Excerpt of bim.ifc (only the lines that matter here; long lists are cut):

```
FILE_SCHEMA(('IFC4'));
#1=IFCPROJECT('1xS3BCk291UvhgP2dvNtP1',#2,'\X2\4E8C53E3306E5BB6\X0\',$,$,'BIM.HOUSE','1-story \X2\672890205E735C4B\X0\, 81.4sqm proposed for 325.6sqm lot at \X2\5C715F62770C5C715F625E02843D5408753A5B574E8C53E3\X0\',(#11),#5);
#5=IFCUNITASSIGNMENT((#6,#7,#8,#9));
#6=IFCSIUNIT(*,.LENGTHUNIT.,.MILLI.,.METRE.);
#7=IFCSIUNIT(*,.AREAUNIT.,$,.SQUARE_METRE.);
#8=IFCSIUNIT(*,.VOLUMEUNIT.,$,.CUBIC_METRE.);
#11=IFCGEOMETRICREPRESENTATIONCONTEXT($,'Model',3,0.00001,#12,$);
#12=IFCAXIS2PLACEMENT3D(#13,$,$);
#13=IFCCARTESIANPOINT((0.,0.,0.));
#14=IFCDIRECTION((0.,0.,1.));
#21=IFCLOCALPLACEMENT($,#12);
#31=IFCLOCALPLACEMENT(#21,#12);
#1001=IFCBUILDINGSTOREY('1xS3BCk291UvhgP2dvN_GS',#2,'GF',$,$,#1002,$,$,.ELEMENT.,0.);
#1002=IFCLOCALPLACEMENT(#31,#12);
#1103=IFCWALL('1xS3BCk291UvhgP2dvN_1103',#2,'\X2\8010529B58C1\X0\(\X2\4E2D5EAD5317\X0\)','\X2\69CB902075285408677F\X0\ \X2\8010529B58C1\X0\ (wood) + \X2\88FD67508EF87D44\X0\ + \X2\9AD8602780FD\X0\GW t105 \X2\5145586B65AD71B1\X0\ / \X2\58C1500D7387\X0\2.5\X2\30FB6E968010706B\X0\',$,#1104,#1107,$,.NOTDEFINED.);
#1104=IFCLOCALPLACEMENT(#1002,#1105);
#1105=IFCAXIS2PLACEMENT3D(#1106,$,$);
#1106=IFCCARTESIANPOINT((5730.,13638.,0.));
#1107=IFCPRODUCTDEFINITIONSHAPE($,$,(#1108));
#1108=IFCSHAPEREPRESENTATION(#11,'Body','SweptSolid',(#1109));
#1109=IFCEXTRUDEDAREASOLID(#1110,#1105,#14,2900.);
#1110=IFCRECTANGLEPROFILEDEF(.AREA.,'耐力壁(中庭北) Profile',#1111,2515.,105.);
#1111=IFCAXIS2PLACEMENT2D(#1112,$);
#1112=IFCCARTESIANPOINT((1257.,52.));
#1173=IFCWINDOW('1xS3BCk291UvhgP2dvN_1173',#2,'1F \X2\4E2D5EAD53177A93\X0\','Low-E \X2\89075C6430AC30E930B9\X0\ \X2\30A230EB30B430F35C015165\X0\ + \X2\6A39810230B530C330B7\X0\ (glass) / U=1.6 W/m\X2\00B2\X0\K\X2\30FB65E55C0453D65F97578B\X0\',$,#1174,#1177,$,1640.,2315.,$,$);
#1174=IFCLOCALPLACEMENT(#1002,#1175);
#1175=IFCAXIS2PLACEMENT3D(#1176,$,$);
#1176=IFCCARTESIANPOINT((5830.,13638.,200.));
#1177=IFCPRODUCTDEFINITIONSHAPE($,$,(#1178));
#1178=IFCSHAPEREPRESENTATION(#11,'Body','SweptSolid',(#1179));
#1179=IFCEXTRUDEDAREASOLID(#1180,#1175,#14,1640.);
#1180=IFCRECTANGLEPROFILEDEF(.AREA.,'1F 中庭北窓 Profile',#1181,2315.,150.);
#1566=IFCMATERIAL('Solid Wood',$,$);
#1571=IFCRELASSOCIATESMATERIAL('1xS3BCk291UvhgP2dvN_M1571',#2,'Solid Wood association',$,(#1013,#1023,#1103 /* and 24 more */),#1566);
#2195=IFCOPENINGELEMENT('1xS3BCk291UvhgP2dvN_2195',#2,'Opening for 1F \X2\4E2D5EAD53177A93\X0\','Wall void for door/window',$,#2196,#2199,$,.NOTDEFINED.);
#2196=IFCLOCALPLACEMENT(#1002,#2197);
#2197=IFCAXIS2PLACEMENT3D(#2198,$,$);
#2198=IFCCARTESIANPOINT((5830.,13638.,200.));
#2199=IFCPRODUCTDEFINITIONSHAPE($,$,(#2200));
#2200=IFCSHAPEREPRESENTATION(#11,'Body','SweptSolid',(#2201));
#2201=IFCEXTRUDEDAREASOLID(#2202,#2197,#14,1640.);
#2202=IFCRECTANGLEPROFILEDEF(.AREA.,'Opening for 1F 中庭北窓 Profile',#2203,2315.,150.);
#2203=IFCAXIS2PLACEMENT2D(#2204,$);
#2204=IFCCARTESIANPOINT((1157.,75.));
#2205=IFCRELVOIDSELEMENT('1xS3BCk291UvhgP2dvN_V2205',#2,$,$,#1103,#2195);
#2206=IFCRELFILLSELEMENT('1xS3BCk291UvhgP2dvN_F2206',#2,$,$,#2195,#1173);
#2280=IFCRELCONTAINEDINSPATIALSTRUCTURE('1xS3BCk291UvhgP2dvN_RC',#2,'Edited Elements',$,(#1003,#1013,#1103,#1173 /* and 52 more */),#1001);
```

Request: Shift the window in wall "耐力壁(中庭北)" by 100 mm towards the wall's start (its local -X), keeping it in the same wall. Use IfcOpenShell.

```python
import ifcopenshell
import ifcopenshell.api.geometry
import ifcopenshell.util.placement

model = ifcopenshell.open("bim.ifc")

window = model.by_guid("1xS3BCk291UvhgP2dvN_1173")
opening = window.FillsVoids[0].RelatingOpeningElement
wall = opening.VoidsElements[0].RelatingBuildingElement

wall_matrix = ifcopenshell.util.placement.get_local_placement(wall.ObjectPlacement)
shift = wall_matrix[:3, 0] * -100.0
before = ifcopenshell.util.placement.get_local_placement(window.ObjectPlacement)[:3, 3].copy()

# The window is not placed relative to its opening, so move both.
for product in (opening, window):
    matrix = ifcopenshell.util.placement.get_local_placement(product.ObjectPlacement)
    matrix[:3, 3] += shift
    ifcopenshell.api.geometry.edit_object_placement(model, product=product, matrix=matrix, is_si=False)

after = ifcopenshell.util.placement.get_local_placement(window.ObjectPlacement)[:3, 3]
print("window moved by", (after - before).round(3) + 0.0)

model.write("bim_rev.ifc")
```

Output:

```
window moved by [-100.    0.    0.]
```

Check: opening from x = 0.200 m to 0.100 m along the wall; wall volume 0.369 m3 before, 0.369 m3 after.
